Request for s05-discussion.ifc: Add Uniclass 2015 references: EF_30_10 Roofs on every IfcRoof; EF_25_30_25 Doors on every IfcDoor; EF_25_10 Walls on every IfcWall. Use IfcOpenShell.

First a look at what the model holds.

```python
import ifcopenshell

model = ifcopenshell.open("s05-discussion.ifc")
print(model.schema)
print("classifications:", [c.Name for c in model.by_type("IfcClassification")])
for ifc_class in ("IfcDoor", "IfcRoof", "IfcStair", "IfcWall", "IfcWindow"):
    print(ifc_class, len(model.by_type(ifc_class)))
```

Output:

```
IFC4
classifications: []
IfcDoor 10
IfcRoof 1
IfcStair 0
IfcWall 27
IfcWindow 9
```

```python
import ifcopenshell
import ifcopenshell.api.classification

model = ifcopenshell.open("s05-discussion.ifc")

system = ifcopenshell.api.classification.add_classification(model, classification="Uniclass 2015")

codes = {
    "IfcRoof": ("EF_30_10", "Roofs"),
    "IfcDoor": ("EF_25_30_25", "Doors"),
    "IfcWall": ("EF_25_10", "Walls"),
}
for ifc_class, (code, name) in codes.items():
    products = model.by_type(ifc_class)
    ifcopenshell.api.classification.add_reference(
        model, products=products, classification=system, identification=code, name=name
    )
    print(code, len(products))

model.write("s05-discussion-out.ifc")
```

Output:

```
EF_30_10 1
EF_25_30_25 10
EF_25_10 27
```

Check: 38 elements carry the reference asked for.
